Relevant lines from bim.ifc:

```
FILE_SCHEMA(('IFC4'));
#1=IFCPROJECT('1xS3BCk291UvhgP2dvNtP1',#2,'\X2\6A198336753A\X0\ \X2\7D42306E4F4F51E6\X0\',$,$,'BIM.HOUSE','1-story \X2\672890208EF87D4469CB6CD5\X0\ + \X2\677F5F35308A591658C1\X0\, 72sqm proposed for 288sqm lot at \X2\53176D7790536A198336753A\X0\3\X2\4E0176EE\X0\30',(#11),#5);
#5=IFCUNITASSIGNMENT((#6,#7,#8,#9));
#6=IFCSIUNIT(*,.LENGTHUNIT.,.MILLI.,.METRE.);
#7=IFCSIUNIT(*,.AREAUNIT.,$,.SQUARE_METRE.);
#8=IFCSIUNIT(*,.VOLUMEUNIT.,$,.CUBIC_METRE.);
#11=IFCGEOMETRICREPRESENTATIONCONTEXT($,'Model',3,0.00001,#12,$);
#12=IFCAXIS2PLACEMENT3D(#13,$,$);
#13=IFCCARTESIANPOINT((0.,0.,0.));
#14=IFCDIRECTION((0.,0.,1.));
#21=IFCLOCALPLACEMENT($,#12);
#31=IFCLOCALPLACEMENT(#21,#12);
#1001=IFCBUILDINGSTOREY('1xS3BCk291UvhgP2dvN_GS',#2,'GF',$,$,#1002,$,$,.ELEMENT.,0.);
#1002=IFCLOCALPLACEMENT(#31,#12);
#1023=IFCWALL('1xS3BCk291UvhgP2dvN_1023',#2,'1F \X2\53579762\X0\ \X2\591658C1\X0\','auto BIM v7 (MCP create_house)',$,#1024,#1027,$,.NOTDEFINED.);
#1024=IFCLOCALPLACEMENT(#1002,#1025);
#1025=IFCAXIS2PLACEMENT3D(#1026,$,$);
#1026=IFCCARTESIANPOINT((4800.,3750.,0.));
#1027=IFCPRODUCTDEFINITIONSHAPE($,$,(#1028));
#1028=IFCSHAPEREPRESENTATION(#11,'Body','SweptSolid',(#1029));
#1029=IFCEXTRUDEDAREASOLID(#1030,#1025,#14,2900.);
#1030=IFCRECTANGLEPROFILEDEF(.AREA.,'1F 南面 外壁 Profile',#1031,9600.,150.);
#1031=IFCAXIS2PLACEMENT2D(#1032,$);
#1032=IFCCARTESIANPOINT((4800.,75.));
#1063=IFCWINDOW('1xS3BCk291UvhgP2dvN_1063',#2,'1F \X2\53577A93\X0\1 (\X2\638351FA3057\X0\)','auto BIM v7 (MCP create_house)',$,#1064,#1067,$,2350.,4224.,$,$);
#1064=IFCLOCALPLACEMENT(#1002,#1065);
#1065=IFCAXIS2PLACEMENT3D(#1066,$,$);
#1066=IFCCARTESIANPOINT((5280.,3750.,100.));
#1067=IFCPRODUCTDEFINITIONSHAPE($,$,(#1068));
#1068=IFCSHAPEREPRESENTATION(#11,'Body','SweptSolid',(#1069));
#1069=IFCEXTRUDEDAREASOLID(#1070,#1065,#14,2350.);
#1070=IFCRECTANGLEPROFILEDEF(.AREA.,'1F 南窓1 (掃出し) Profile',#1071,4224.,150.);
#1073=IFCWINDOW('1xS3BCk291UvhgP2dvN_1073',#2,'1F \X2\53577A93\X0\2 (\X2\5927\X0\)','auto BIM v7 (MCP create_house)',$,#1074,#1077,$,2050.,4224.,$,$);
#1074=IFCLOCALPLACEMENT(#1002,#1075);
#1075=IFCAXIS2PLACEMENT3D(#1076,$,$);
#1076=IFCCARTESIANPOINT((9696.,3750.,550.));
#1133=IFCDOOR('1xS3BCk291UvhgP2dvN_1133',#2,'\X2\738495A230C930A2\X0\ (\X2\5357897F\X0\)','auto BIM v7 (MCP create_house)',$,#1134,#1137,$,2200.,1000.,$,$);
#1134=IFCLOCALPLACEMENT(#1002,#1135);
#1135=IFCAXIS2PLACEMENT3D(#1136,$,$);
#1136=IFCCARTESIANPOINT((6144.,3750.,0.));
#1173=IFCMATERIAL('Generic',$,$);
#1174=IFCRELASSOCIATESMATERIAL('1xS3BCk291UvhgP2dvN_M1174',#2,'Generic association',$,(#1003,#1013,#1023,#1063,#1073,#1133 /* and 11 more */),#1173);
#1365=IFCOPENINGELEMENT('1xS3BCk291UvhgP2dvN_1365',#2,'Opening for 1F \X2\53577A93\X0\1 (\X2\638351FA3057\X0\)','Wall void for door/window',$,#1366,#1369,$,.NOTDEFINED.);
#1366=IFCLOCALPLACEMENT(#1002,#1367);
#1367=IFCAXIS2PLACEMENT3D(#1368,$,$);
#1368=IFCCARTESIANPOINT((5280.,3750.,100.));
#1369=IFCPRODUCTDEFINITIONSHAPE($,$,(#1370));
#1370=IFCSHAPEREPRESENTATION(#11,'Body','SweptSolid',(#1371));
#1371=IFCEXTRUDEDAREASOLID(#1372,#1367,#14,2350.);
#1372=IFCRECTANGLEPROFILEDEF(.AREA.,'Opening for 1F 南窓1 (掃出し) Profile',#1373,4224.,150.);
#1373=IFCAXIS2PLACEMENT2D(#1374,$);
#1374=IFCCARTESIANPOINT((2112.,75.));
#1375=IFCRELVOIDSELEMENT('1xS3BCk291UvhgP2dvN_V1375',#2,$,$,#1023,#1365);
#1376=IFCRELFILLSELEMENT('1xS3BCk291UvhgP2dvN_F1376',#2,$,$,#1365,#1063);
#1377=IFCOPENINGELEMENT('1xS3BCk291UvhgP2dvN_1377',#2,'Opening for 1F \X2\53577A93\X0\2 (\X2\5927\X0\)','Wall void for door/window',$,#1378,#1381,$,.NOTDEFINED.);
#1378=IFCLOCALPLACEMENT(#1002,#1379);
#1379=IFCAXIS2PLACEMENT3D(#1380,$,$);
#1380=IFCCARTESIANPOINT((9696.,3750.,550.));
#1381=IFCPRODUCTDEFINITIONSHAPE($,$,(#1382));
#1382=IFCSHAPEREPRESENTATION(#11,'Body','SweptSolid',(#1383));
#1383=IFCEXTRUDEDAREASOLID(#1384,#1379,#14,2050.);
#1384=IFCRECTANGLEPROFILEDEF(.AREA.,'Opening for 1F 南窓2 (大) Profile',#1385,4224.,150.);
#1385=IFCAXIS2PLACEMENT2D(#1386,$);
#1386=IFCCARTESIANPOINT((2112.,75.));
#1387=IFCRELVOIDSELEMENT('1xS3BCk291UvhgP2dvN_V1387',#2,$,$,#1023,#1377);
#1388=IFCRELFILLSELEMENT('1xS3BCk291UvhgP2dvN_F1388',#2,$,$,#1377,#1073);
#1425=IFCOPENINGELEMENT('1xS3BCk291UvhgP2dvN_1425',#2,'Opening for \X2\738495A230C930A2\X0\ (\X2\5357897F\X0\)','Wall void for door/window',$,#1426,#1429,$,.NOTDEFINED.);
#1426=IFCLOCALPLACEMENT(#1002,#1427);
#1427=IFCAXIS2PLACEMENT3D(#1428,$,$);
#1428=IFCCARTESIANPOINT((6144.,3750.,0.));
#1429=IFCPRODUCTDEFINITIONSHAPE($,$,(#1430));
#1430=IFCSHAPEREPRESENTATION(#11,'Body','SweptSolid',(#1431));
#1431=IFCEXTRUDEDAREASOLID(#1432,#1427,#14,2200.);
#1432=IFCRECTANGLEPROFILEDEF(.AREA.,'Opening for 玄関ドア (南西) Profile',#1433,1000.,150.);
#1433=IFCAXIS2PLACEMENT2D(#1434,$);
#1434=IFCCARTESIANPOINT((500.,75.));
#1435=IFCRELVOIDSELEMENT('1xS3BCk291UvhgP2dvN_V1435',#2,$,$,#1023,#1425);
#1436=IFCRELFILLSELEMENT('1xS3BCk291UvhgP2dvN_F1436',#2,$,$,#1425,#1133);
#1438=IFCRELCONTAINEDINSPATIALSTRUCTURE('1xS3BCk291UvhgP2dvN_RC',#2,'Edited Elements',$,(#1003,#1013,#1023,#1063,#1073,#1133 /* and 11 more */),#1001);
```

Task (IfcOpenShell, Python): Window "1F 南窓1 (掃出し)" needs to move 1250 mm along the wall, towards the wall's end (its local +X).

```python
import ifcopenshell
import ifcopenshell.api.geometry
import ifcopenshell.util.placement

model = ifcopenshell.open("bim.ifc")

window = model.by_guid("1xS3BCk291UvhgP2dvN_1063")
opening = window.FillsVoids[0].RelatingOpeningElement
wall = opening.VoidsElements[0].RelatingBuildingElement

wall_matrix = ifcopenshell.util.placement.get_local_placement(wall.ObjectPlacement)
shift = wall_matrix[:3, 0] * 1250.0
before = ifcopenshell.util.placement.get_local_placement(window.ObjectPlacement)[:3, 3].copy()

# The window is not placed relative to its opening, so move both.
for product in (opening, window):
    matrix = ifcopenshell.util.placement.get_local_placement(product.ObjectPlacement)
    matrix[:3, 3] += shift
    ifcopenshell.api.geometry.edit_object_placement(model, product=product, matrix=matrix, is_si=False)

after = ifcopenshell.util.placement.get_local_placement(window.ObjectPlacement)[:3, 3]
print("window moved by", (after - before).round(3) + 0.0)

model.write("bim_v2.ifc")
```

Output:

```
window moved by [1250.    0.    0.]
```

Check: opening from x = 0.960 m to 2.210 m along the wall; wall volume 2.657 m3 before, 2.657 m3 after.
